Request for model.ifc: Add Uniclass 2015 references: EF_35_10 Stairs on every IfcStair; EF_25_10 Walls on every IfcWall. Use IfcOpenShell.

First a look at what the model holds.

```python
import ifcopenshell

model = ifcopenshell.open("model.ifc")
print(model.schema)
print("classifications:", [c.Name for c in model.by_type("IfcClassification")])
for ifc_class in ("IfcDoor", "IfcRoof", "IfcStair", "IfcWall", "IfcWindow"):
    print(ifc_class, len(model.by_type(ifc_class)))
```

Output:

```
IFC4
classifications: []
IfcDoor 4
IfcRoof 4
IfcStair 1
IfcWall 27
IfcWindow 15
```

```python
import ifcopenshell
import ifcopenshell.api.classification

model = ifcopenshell.open("model.ifc")

system = ifcopenshell.api.classification.add_classification(model, classification="Uniclass 2015")

codes = {
    "IfcStair": ("EF_35_10", "Stairs"),
    "IfcWall": ("EF_25_10", "Walls"),
}
for ifc_class, (code, name) in codes.items():
    products = model.by_type(ifc_class)
    ifcopenshell.api.classification.add_reference(
        model, products=products, classification=system, identification=code, name=name
    )
    print(code, len(products))

model.write("model-out.ifc")
```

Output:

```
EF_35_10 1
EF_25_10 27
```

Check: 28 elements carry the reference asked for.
